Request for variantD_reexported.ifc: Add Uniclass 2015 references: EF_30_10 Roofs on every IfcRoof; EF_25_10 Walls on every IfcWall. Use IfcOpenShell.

First a look at what the model holds.

```python
import ifcopenshell

model = ifcopenshell.open("variantD_reexported.ifc")
print(model.schema)
print("classifications:", [c.Name for c in model.by_type("IfcClassification")])
for ifc_class in ("IfcDoor", "IfcRoof", "IfcStair", "IfcWall", "IfcWindow"):
    print(ifc_class, len(model.by_type(ifc_class)))
```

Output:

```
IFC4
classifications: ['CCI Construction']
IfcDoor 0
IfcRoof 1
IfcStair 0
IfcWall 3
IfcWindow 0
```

```python
import ifcopenshell
import ifcopenshell.api.classification

model = ifcopenshell.open("variantD_reexported.ifc")

system = ifcopenshell.api.classification.add_classification(model, classification="Uniclass 2015")

codes = {
    "IfcRoof": ("EF_30_10", "Roofs"),
    "IfcWall": ("EF_25_10", "Walls"),
}
for ifc_class, (code, name) in codes.items():
    products = model.by_type(ifc_class)
    ifcopenshell.api.classification.add_reference(
        model, products=products, classification=system, identification=code, name=name
    )
    print(code, len(products))

model.write("variantD_reexported_edited.ifc")
```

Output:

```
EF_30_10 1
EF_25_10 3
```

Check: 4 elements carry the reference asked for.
